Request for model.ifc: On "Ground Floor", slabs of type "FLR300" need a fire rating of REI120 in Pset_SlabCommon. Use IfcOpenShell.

First a look at what the model holds.

```python
import ifcopenshell
import ifcopenshell.util.element

model = ifcopenshell.open("model.ifc")
print(model.schema)
storey = next(s for s in model.by_type("IfcBuildingStorey") if s.Name == "Ground Floor")
slabs = [e for e in ifcopenshell.util.element.get_decomposition(storey) if e.is_a("IfcSlab")]
seen = {}
for e in slabs:
    element_type = ifcopenshell.util.element.get_type(e)
    key = (element_type.Name if element_type != e and element_type else None, ifcopenshell.util.element.get_pset(e, "Pset_SlabCommon", "FireRating"))
    seen[key] = seen.get(key, 0) + 1
for (name, value), count in sorted(seen.items(), key=str):
    print(count, "x", name, "|", value)
```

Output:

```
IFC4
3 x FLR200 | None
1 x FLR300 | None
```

```python
import ifcopenshell
import ifcopenshell.api.pset
import ifcopenshell.util.element

model = ifcopenshell.open("model.ifc")

storey = next(s for s in model.by_type("IfcBuildingStorey") if s.Name == "Ground Floor")
slabs = [e for e in ifcopenshell.util.element.get_decomposition(storey) if e.is_a("IfcSlab")]

count = 0
for e in slabs:
    element_type = ifcopenshell.util.element.get_type(e)
    if element_type in (None, e) or element_type.Name != "FLR300":
        continue
    # add_pset returns the element's existing set when there is one.
    pset = ifcopenshell.api.pset.add_pset(model, product=e, name="Pset_SlabCommon")
    ifcopenshell.api.pset.edit_pset(model, pset=pset, properties={"FireRating": "REI120"})
    count += 1

print(count, "slabs updated")

model.write("model_edited.ifc")
```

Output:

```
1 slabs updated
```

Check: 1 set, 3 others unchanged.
